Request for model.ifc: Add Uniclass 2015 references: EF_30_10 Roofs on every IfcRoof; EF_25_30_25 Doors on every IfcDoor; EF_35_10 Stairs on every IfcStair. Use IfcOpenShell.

First a look at what the model holds.

```python
import ifcopenshell

model = ifcopenshell.open("model.ifc")
print(model.schema)
print("classifications:", [c.Name for c in model.by_type("IfcClassification")])
for ifc_class in ("IfcDoor", "IfcRoof", "IfcStair", "IfcWall", "IfcWindow"):
    print(ifc_class, len(model.by_type(ifc_class)))
```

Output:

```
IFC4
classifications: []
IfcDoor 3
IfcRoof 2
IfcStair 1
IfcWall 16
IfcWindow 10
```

```python
import ifcopenshell
import ifcopenshell.api.classification

model = ifcopenshell.open("model.ifc")

system = ifcopenshell.api.classification.add_classification(model, classification="Uniclass 2015")

codes = {
    "IfcRoof": ("EF_30_10", "Roofs"),
    "IfcDoor": ("EF_25_30_25", "Doors"),
    "IfcStair": ("EF_35_10", "Stairs"),
}
for ifc_class, (code, name) in codes.items():
    products = model.by_type(ifc_class)
    ifcopenshell.api.classification.add_reference(
        model, products=products, classification=system, identification=code, name=name
    )
    print(code, len(products))

model.write("model_edited.ifc")
```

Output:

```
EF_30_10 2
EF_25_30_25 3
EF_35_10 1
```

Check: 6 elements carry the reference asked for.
